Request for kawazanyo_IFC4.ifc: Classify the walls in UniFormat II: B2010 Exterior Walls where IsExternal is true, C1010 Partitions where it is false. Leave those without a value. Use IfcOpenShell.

First a look at what the model holds.

```python
import ifcopenshell
import ifcopenshell.util.element

model = ifcopenshell.open("kawazanyo_IFC4.ifc")
print(model.schema)
print("classifications:", [c.Name for c in model.by_type("IfcClassification")])
values = [ifcopenshell.util.element.get_pset(e, "Pset_WallCommon", "IsExternal") for e in model.by_type("IfcWall")]
for value in (True, False, None):
    print("IsExternal", value, values.count(value))
```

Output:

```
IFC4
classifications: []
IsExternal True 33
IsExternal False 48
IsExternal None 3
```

```python
import ifcopenshell
import ifcopenshell.api.classification
import ifcopenshell.util.element

model = ifcopenshell.open("kawazanyo_IFC4.ifc")

system = ifcopenshell.api.classification.add_classification(model, classification="UniFormat II")

walls = model.by_type("IfcWall")
external = {e: ifcopenshell.util.element.get_pset(e, "Pset_WallCommon", "IsExternal") for e in walls}
for flag, code, name in ((True, "B2010", "Exterior Walls"), (False, "C1010", "Partitions")):
    products = [e for e in walls if external[e] is flag]
    ifcopenshell.api.classification.add_reference(
        model, products=products, classification=system, identification=code, name=name
    )
    print(code, len(products))

model.write("kawazanyo_IFC4_v2.ifc")
```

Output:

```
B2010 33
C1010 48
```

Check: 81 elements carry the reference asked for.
